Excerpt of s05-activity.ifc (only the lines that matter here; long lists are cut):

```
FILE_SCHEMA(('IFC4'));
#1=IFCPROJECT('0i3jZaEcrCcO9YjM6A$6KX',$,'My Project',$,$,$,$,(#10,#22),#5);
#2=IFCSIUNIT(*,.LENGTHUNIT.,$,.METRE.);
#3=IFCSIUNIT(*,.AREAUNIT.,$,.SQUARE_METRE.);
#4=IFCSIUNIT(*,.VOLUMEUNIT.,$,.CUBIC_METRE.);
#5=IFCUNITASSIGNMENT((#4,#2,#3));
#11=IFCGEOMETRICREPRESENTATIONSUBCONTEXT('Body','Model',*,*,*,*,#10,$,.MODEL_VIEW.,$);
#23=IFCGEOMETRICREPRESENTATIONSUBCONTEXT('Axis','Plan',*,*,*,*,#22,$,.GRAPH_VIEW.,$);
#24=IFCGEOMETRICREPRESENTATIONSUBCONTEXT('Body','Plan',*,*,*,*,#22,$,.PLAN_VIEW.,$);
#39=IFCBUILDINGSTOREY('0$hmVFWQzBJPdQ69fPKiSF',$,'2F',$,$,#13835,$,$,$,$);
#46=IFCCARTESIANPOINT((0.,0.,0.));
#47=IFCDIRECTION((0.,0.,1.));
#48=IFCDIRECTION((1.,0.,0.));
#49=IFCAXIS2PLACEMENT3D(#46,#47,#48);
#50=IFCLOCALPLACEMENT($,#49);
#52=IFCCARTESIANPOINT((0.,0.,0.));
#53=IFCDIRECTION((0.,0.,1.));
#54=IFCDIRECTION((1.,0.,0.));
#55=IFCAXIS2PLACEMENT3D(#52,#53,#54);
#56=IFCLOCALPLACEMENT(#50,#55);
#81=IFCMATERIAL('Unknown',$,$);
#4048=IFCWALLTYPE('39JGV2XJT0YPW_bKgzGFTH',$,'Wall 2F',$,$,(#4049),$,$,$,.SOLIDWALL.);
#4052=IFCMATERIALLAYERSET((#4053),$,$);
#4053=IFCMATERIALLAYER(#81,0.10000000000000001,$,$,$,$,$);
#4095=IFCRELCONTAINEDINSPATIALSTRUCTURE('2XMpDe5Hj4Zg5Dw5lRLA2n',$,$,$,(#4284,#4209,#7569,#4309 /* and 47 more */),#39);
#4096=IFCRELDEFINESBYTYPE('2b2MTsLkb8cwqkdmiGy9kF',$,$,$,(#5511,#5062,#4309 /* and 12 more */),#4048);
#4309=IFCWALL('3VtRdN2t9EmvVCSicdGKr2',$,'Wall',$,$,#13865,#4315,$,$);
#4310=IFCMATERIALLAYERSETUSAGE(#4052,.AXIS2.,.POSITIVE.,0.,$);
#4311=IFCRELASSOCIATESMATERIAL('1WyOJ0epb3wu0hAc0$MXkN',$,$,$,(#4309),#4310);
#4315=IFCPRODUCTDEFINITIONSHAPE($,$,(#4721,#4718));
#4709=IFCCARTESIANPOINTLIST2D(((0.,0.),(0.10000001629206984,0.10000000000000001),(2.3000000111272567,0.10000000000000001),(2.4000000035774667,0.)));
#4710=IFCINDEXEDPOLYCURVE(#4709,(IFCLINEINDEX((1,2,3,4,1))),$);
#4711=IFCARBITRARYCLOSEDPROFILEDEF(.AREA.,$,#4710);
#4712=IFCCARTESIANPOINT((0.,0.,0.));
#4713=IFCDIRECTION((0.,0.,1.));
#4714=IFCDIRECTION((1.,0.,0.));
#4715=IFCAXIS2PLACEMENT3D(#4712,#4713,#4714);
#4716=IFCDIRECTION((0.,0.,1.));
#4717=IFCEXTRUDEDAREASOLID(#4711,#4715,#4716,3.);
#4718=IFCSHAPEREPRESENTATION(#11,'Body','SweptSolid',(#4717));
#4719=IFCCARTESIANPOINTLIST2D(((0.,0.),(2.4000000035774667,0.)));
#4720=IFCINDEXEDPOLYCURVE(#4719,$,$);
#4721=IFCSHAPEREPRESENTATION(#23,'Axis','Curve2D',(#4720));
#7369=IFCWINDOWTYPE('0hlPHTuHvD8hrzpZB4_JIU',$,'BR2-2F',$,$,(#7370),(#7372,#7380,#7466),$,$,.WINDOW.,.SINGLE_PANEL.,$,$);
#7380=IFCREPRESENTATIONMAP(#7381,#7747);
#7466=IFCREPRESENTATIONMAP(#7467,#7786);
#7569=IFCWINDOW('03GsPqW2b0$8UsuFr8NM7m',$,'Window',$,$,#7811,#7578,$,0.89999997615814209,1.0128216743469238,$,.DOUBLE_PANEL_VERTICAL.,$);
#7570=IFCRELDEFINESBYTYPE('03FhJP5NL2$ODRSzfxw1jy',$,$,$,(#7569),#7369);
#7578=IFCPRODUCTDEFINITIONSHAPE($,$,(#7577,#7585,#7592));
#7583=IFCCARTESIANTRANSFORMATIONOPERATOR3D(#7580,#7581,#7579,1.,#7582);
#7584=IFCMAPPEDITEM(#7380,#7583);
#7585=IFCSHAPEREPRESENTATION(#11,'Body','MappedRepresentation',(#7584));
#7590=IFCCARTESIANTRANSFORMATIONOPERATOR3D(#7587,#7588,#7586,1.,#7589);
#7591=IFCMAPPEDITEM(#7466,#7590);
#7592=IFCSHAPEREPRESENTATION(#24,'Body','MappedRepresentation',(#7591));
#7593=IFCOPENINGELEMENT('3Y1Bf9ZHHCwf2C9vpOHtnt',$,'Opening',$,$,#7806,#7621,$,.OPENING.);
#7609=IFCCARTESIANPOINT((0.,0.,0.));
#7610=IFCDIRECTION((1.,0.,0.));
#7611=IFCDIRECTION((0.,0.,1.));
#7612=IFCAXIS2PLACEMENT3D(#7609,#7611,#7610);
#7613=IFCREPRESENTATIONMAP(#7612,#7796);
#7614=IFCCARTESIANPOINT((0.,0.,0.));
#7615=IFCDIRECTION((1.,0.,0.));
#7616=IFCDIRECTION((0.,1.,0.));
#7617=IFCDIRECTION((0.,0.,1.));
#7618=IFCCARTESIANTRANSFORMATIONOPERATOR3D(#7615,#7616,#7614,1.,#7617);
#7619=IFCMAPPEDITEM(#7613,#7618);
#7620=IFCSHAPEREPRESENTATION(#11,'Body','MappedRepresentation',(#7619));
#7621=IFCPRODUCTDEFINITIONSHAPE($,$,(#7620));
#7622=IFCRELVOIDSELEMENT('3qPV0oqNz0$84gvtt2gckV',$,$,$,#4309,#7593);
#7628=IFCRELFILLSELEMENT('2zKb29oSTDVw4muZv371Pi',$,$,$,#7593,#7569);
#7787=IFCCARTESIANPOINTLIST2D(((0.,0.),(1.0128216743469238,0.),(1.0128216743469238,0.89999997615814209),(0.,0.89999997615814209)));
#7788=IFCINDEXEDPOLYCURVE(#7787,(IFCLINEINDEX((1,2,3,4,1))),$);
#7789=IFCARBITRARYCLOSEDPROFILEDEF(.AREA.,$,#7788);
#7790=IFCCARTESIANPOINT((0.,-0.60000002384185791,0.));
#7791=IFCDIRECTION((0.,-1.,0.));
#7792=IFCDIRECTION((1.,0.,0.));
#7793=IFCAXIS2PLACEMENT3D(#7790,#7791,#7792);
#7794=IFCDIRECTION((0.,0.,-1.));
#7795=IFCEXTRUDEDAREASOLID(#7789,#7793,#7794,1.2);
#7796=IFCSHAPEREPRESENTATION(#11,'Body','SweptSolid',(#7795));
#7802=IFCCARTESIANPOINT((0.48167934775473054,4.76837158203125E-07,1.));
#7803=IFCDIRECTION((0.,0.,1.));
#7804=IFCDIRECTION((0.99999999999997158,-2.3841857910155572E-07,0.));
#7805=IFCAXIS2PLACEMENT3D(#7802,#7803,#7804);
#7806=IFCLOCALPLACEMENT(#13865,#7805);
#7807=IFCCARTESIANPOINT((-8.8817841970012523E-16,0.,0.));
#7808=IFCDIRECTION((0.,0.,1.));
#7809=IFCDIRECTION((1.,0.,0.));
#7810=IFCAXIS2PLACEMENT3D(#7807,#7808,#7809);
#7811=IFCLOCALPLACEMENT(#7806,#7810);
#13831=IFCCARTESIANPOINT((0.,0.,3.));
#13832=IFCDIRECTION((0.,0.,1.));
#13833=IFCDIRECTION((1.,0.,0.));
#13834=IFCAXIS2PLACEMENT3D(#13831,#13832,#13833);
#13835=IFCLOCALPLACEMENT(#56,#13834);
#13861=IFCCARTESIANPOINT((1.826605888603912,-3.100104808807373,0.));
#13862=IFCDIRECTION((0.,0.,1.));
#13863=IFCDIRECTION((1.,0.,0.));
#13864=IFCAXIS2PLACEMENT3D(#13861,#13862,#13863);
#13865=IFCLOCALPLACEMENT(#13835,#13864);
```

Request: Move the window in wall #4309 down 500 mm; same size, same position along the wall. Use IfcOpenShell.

```python
import numpy as np
import ifcopenshell
import ifcopenshell.api.geometry
import ifcopenshell.util.placement
import ifcopenshell.util.unit

model = ifcopenshell.open("s05-activity.ifc")
unit_scale = ifcopenshell.util.unit.calculate_unit_scale(model)

window = model.by_id(7569)
opening = window.FillsVoids[0].RelatingOpeningElement
dz = -0.5

shift = np.array([0.0, 0.0, dz])
# The window is placed relative to its opening, so it follows when the opening moves.
matrix = ifcopenshell.util.placement.get_local_placement(opening.ObjectPlacement)
matrix[:3, 3] += shift
ifcopenshell.api.geometry.edit_object_placement(
    model, product=opening, matrix=matrix, is_si=False, should_transform_children=True
)

print(f"moved by {dz * unit_scale:+.3f} m")

model.write("s05-activity_v2.ifc")
```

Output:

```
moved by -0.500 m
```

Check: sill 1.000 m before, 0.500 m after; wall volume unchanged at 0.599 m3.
